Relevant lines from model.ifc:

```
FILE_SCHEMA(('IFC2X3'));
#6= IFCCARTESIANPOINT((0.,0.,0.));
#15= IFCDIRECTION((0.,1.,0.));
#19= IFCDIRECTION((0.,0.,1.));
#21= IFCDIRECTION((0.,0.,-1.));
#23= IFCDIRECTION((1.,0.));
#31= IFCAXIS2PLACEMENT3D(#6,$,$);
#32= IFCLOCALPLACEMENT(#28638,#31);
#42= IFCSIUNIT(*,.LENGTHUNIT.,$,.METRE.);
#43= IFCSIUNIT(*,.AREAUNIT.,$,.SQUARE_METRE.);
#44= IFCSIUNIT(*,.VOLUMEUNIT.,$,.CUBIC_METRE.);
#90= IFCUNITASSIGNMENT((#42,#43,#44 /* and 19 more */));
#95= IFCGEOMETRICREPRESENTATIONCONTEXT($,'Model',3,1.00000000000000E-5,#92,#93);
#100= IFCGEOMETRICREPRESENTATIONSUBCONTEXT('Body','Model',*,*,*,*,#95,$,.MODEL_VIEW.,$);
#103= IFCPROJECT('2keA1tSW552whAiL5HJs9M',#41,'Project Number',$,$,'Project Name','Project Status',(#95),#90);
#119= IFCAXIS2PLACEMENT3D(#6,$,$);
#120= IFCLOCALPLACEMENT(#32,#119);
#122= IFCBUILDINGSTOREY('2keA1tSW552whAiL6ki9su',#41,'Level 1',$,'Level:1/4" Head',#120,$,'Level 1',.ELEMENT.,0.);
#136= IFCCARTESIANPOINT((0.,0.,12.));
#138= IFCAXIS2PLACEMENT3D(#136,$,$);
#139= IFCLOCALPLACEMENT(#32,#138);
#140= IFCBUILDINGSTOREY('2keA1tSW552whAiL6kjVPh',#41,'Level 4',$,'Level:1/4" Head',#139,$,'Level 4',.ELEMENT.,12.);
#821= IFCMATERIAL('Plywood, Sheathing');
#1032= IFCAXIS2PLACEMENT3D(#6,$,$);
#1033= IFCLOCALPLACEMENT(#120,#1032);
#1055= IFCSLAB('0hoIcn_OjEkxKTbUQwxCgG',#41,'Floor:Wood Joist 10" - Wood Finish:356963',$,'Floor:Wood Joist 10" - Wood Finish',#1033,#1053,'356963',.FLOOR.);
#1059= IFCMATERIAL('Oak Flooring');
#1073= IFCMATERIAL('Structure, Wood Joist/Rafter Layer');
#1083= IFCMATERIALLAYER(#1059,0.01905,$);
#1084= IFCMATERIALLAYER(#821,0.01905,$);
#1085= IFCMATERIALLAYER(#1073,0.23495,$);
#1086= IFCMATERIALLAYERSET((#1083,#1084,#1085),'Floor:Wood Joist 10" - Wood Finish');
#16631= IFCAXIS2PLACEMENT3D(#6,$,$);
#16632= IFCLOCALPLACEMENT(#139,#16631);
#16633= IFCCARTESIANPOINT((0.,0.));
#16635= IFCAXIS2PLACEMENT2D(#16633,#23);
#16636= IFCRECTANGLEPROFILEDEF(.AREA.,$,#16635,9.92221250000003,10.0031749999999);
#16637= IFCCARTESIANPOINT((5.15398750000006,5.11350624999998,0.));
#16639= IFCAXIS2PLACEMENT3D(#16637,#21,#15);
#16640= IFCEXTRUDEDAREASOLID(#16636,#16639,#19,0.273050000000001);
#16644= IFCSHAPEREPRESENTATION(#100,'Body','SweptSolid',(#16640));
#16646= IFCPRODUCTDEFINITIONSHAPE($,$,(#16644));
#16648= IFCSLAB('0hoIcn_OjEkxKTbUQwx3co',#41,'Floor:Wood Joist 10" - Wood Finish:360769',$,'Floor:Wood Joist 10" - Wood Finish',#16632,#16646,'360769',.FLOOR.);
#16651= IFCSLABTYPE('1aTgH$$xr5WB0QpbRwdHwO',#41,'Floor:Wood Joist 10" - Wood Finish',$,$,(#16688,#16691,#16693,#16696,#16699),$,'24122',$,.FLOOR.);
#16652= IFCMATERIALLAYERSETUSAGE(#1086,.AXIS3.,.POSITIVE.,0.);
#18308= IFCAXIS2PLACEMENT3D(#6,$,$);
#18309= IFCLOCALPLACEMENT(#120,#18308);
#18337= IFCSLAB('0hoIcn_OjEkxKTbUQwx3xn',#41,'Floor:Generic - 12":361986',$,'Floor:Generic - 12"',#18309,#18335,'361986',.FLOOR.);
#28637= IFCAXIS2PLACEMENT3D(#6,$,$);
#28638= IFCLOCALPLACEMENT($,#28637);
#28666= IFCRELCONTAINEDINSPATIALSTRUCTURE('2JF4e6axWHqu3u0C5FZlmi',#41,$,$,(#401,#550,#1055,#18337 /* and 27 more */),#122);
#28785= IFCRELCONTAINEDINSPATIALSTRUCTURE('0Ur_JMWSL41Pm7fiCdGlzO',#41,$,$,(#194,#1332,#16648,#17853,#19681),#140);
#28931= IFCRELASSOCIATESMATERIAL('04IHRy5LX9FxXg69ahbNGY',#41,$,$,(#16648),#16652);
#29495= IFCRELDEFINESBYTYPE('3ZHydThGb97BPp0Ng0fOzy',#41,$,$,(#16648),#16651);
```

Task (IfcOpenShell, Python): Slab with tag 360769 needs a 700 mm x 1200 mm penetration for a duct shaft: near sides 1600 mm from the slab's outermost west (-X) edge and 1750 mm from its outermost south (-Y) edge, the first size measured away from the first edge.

```python
import numpy as np
import ifcopenshell
import ifcopenshell.api.feature
import ifcopenshell.api.geometry
import ifcopenshell.api.root
import ifcopenshell.geom
import ifcopenshell.util.placement
import ifcopenshell.util.representation
import ifcopenshell.util.shape
import ifcopenshell.util.unit

model = ifcopenshell.open("model.ifc")
unit_scale = ifcopenshell.util.unit.calculate_unit_scale(model)
settings = ifcopenshell.geom.settings()


def volume(element):
    """Net volume in cubic metres, openings subtracted."""
    shape = ifcopenshell.geom.create_shape(settings, element)
    return ifcopenshell.util.shape.get_volume(shape.geometry)


slab = model.by_guid("0hoIcn_OjEkxKTbUQwx3co")
before = volume(slab)

# Extent in the slab's own axes, in metres. The edges named are its -X and -Y sides.
slab_shape = ifcopenshell.geom.create_shape(settings, slab)
vertices = ifcopenshell.util.shape.get_vertices(slab_shape.geometry)
x_min, y_min, bottom = vertices.min(axis=0)
top = vertices[:, 2].max()

opening = ifcopenshell.api.root.create_entity(model, ifc_class="IfcOpeningElement", name="Duct shaft opening")
context = ifcopenshell.util.representation.get_context(model, "Model", "Body", "MODEL_VIEW")
width, depth = 0.7, 1.2
outline = [(0.0, 0.0), (width, 0.0), (width, depth), (0.0, depth), (0.0, 0.0)]
# Overshoot both faces by 50 mm so the cut is clean.
shape = ifcopenshell.api.geometry.add_slab_representation(
    model, context=context, depth=top - bottom + 0.1, polyline=outline
)
ifcopenshell.api.geometry.assign_representation(model, product=opening, representation=shape)

matrix = ifcopenshell.util.placement.get_local_placement(slab.ObjectPlacement)
matrix[:, 3] = matrix @ np.append(np.array([x_min + 1.6, y_min + 1.75, bottom - 0.05]) / unit_scale, 1.0)
ifcopenshell.api.geometry.edit_object_placement(model, product=opening, matrix=matrix, is_si=False)
ifcopenshell.api.feature.add_feature(model, feature=opening, element=slab)

after = volume(slab)

print(f"slab volume {before:.3f} -> {after:.3f} m3")

model.write("model_edited.ifc")
```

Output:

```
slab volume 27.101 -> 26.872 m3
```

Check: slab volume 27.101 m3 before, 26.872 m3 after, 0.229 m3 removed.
